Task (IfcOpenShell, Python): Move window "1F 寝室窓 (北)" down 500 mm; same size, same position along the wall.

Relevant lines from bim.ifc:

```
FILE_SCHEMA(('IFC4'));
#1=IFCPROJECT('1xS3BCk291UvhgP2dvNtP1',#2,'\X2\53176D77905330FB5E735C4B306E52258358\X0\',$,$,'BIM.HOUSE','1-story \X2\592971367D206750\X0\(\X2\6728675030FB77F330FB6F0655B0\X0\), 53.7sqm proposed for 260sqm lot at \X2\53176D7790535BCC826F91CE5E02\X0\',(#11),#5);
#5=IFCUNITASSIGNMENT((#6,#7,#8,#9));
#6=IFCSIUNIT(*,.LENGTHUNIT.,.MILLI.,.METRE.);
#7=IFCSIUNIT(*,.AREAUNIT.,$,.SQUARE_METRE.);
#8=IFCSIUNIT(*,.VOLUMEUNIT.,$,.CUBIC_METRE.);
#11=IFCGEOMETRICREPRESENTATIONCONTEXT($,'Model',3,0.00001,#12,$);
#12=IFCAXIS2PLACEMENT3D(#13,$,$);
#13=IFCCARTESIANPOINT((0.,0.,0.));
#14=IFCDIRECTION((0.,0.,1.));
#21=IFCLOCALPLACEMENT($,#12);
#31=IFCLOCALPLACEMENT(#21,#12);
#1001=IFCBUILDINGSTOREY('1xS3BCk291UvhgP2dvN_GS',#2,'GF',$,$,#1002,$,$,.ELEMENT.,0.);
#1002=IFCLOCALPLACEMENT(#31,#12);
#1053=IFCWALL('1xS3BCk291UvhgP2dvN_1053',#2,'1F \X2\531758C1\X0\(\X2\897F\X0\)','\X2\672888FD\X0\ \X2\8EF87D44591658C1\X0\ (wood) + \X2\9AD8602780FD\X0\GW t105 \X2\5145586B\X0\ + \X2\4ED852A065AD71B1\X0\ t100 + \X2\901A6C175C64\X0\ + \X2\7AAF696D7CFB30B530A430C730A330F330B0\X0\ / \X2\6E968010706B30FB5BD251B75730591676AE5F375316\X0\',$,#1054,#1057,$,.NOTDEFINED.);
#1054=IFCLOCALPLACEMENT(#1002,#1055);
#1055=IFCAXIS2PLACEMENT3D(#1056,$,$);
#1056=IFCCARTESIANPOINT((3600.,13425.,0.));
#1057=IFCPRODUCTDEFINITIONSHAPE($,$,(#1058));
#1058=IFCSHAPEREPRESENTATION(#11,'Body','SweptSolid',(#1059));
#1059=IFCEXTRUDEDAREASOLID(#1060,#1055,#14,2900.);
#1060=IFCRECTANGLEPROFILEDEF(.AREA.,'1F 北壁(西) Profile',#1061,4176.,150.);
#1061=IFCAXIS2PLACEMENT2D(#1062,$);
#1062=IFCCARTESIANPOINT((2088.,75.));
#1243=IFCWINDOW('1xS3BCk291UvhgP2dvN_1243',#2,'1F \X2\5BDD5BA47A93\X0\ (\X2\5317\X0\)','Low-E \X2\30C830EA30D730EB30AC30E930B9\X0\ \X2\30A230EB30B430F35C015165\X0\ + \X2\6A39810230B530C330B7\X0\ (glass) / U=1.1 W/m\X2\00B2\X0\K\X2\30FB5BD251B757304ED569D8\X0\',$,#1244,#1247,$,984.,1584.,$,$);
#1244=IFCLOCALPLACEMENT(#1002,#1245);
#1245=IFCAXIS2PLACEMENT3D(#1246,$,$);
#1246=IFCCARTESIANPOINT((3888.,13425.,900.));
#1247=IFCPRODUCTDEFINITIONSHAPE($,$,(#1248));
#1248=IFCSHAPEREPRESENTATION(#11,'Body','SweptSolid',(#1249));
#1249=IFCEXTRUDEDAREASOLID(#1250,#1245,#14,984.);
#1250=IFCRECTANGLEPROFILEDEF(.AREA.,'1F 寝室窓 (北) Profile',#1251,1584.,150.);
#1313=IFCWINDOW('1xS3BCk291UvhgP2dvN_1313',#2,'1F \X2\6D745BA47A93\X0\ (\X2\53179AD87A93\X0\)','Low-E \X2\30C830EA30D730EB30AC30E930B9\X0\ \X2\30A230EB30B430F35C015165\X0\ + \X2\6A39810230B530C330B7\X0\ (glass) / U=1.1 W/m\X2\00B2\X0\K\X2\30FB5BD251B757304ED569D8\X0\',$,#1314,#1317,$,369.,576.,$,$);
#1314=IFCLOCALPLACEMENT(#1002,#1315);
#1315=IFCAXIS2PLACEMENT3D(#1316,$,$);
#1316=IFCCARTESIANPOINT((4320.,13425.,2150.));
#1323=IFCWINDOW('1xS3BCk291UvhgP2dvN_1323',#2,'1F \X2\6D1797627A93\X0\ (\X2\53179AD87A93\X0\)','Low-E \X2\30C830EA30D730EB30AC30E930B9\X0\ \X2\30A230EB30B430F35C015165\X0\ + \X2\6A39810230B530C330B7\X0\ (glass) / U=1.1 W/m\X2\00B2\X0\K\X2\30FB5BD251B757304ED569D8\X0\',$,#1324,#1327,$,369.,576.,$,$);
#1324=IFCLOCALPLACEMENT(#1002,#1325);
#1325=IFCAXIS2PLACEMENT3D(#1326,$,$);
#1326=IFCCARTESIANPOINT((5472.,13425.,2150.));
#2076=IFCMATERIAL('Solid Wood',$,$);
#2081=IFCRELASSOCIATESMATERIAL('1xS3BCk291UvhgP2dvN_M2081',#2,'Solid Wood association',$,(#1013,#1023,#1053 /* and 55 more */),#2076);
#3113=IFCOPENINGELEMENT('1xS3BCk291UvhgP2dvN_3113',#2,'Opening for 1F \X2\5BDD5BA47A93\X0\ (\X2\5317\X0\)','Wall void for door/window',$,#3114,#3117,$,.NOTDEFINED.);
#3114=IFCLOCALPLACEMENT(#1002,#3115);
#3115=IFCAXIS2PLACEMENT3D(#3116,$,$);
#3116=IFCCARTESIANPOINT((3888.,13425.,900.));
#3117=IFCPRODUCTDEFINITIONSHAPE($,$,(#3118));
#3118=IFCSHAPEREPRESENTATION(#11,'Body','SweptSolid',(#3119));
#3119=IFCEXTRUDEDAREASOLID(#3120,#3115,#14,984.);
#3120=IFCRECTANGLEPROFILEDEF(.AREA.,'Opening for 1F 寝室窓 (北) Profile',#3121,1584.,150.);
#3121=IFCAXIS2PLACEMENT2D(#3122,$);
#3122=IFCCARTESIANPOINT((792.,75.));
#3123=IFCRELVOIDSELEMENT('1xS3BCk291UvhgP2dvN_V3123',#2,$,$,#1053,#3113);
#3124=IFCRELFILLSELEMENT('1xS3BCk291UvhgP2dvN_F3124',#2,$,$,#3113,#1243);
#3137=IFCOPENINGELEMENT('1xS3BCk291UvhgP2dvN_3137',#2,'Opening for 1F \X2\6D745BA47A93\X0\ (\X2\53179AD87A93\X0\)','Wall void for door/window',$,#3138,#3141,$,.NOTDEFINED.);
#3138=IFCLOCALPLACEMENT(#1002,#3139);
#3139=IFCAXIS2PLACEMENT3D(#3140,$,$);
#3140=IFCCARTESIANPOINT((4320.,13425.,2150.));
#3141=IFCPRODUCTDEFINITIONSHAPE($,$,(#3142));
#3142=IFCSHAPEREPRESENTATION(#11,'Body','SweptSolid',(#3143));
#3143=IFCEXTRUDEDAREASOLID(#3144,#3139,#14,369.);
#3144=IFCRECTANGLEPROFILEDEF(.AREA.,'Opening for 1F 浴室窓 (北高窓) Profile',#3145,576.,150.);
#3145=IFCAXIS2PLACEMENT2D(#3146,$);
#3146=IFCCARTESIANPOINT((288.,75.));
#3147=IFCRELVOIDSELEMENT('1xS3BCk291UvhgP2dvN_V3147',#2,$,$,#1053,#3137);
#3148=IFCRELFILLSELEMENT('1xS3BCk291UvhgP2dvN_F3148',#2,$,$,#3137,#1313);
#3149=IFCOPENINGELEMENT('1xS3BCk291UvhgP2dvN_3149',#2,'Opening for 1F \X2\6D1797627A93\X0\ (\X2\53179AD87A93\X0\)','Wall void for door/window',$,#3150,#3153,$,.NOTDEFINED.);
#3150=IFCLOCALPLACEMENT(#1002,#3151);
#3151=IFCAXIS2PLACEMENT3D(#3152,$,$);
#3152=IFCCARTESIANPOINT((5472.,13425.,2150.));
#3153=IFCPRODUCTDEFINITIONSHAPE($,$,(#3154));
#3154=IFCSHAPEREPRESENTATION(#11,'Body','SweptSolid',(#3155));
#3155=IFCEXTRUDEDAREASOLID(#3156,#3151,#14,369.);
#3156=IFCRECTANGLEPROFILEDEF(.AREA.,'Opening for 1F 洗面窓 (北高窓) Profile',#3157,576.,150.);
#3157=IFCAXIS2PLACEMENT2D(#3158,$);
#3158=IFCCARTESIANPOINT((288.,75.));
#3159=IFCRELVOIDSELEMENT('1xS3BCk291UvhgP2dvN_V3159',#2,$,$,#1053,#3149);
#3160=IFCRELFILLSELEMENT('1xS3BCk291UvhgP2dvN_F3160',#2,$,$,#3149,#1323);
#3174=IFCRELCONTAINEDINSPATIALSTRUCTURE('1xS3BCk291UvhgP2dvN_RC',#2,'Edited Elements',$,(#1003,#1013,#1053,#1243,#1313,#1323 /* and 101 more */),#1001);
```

```python
import numpy as np
import ifcopenshell
import ifcopenshell.api.geometry
import ifcopenshell.util.placement
import ifcopenshell.util.unit

model = ifcopenshell.open("bim.ifc")
unit_scale = ifcopenshell.util.unit.calculate_unit_scale(model)

window = model.by_guid("1xS3BCk291UvhgP2dvN_1243")
opening = window.FillsVoids[0].RelatingOpeningElement
dz = -0.5 / unit_scale

shift = np.array([0.0, 0.0, dz])
# The window is not placed relative to its opening, so move both.
for product in (opening, window):
    matrix = ifcopenshell.util.placement.get_local_placement(product.ObjectPlacement)
    matrix[:3, 3] += shift
    ifcopenshell.api.geometry.edit_object_placement(model, product=product, matrix=matrix, is_si=False)

print(f"moved by {dz * unit_scale:+.3f} m")

model.write("bim_v2.ifc")
```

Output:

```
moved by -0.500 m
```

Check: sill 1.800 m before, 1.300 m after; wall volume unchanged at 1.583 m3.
